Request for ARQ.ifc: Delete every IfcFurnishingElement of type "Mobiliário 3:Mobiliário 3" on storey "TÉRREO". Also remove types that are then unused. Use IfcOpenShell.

First a look at what the model holds.

```python
import ifcopenshell
import ifcopenshell.util.element

model = ifcopenshell.open("ARQ.ifc")
print(model.schema)
storey = next(s for s in model.by_type("IfcBuildingStorey") if s.Name == "TÉRREO")
furniture = [e for e in ifcopenshell.util.element.get_decomposition(storey) if e.is_a("IfcFurnishingElement")]
seen = {}
for e in furniture:
    element_type = ifcopenshell.util.element.get_type(e)
    name = element_type.Name if element_type not in (None, e) else None
    seen[name] = seen.get(name, 0) + 1
for name, count in sorted(seen.items(), key=str):
    print(count, "x", name)
```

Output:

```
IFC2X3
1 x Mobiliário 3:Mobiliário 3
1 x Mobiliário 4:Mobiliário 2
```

```python
import ifcopenshell
import ifcopenshell.api.root
import ifcopenshell.util.element

model = ifcopenshell.open("ARQ.ifc")

storey = next(s for s in model.by_type("IfcBuildingStorey") if s.Name == "TÉRREO")
furniture = [e for e in ifcopenshell.util.element.get_decomposition(storey) if e.is_a("IfcFurnishingElement")]
targets = [e for e in furniture if (t := ifcopenshell.util.element.get_type(e)) not in (None, e) and t.Name == "Mobiliário 3:Mobiliário 3"]
types = {ifcopenshell.util.element.get_type(e) for e in targets} - {None, *targets}

for e in targets:
    ifcopenshell.api.root.remove_product(model, product=e)
print(len(targets), "removed")

unused = [t for t in types if not ifcopenshell.util.element.get_types(t)]
for t in unused:
    ifcopenshell.api.root.remove_product(model, product=t)
print(len(unused), "unused types removed")

model.write("ARQ_rev.ifc")
```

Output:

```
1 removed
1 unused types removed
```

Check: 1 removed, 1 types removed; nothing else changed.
